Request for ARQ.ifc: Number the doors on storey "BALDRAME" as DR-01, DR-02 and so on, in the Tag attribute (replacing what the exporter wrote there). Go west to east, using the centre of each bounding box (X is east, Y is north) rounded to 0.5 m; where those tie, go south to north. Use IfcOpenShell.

First a look at what the model holds.

```python
import ifcopenshell
import ifcopenshell.util.element
import ifcopenshell.util.placement

model = ifcopenshell.open("ARQ.ifc")
print(model.schema)
storey = next(s for s in model.by_type("IfcBuildingStorey") if s.Name == "BALDRAME")
doors = [e for e in ifcopenshell.util.element.get_decomposition(storey) if e.is_a("IfcDoor")]
for e in sorted(doors, key=lambda e: e.id()):
    origin = ifcopenshell.util.placement.get_local_placement(e.ObjectPlacement)[:3, 3]
    print(e.id(), e.Tag, e.Name, origin.round(2) + 0.0, sep=" | ")
```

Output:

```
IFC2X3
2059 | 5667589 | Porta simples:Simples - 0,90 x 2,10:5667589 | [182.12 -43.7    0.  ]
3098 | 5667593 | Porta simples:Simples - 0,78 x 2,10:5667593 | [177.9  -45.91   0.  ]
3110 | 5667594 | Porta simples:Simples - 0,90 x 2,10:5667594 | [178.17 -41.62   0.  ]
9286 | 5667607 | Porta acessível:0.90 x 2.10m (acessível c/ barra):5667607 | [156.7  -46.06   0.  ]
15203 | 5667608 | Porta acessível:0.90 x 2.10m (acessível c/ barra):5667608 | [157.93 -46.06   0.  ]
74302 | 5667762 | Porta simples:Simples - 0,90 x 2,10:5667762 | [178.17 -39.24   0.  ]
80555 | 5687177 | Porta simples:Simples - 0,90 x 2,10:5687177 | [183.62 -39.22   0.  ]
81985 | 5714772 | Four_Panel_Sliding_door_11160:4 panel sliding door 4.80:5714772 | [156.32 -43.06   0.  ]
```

```python
import ifcopenshell
import ifcopenshell.geom
import ifcopenshell.util.element
import ifcopenshell.util.shape

model = ifcopenshell.open("ARQ.ifc")
settings = ifcopenshell.geom.settings()
settings.set("use-world-coords", True)


def centre(element):
    shape = ifcopenshell.geom.create_shape(settings, element)
    return ifcopenshell.util.shape.get_bbox_centroid(shape.geometry)


storey = next(s for s in model.by_type("IfcBuildingStorey") if s.Name == "BALDRAME")
doors = [e for e in ifcopenshell.util.element.get_decomposition(storey) if e.is_a("IfcDoor")]

# Insertion points can sit at a corner or the storey origin, so sort by the geometry (in metres).
centres = {e: centre(e) for e in doors}
doors.sort(key=lambda e: (round(centres[e][0] / 0.5), centres[e][1]))

for i, e in enumerate(doors, start=1):
    number = f"DR-{i:02d}"
    e.Tag = number
    print(e.id(), number)

model.write("ARQ_rev.ifc")
```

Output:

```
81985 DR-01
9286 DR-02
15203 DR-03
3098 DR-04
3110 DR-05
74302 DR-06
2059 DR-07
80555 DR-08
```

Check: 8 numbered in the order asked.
